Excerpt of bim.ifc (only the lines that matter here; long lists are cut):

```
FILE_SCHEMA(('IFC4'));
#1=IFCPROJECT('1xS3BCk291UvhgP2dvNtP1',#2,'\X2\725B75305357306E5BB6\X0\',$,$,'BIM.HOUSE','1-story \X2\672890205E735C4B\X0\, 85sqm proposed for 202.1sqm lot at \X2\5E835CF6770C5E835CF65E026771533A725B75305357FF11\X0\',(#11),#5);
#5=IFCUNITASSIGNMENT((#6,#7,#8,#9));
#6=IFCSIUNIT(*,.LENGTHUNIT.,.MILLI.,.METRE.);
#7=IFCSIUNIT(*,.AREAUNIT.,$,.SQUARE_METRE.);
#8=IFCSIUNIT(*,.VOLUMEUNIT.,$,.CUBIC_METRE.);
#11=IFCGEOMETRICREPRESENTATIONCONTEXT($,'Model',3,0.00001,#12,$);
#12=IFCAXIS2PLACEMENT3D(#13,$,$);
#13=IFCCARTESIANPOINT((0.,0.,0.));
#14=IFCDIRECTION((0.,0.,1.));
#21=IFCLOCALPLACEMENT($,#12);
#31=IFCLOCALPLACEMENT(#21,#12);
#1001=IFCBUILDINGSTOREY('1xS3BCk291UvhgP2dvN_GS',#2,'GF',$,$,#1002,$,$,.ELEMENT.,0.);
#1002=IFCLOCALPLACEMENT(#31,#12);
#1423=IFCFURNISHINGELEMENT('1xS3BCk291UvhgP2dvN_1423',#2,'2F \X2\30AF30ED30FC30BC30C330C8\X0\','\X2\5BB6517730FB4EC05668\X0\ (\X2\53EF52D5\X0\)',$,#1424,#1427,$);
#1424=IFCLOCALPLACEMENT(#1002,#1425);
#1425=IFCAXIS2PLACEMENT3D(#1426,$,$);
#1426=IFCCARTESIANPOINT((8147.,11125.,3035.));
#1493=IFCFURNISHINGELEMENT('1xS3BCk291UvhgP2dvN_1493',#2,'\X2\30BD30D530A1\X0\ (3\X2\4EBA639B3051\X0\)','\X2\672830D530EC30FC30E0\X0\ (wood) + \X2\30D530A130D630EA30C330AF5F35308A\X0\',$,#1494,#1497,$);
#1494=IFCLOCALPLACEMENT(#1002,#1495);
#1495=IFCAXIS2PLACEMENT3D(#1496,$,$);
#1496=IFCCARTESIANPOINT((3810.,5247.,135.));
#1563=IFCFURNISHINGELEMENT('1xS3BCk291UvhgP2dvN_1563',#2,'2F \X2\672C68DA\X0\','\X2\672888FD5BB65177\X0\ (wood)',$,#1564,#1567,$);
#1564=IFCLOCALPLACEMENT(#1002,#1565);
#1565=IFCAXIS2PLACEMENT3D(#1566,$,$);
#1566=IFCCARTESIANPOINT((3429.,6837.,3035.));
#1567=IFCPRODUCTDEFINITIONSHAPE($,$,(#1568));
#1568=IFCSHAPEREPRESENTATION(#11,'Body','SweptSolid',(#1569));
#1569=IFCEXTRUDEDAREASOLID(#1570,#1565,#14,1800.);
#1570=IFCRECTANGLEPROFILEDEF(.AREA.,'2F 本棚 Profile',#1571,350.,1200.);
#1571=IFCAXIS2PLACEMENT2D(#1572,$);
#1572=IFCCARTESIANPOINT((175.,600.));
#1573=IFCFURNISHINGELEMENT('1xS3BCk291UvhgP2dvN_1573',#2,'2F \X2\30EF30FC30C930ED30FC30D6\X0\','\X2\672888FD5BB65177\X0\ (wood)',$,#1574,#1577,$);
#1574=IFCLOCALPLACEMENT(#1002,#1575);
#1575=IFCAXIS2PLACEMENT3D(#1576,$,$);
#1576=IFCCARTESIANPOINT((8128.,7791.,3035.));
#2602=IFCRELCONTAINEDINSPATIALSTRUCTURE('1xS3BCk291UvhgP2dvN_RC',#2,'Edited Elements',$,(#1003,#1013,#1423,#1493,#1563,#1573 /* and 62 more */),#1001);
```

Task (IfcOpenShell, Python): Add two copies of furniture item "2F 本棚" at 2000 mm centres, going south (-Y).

```python
import numpy as np
import ifcopenshell
import ifcopenshell.api.geometry
import ifcopenshell.api.root
import ifcopenshell.util.element
import ifcopenshell.util.placement

model = ifcopenshell.open("bim.ifc")


def reuse_history(source, copy):
    """copy_class also copies each property set's owner history, people and application; keep the originals."""
    for rel in copy.IsDefinedBy:
        if rel.is_a("IfcRelDefinesByProperties") and (history := rel.RelatingPropertyDefinition.OwnerHistory):
            rel.RelatingPropertyDefinition.OwnerHistory = source.OwnerHistory
            ifcopenshell.util.element.remove_deep2(model, history)


source = model.by_guid("1xS3BCk291UvhgP2dvN_1563")
base = ifcopenshell.util.placement.get_local_placement(source.ObjectPlacement)
step = np.array([0.0, -1.0, 0.0]) * 2000.0

for i in range(1, 3):
    copy = ifcopenshell.api.root.copy_class(model, product=source)
    copy.Representation = ifcopenshell.util.element.copy_deep(
        model, source.Representation, exclude=["IfcGeometricRepresentationContext", "IfcRepresentationMap"]
    )
    reuse_history(source, copy)
    matrix = base.copy()
    matrix[:3, 3] += i * step
    print("added at", matrix[:3, 3].round(3) + 0.0)
    ifcopenshell.api.geometry.edit_object_placement(model, product=copy, matrix=matrix, is_si=False)

model.write("bim_rev.ifc")
```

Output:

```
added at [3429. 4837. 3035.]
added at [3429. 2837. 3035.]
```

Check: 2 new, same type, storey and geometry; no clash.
